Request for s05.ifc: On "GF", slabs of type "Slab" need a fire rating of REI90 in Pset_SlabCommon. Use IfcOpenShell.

First a look at what the model holds.

```python
import ifcopenshell
import ifcopenshell.util.element

model = ifcopenshell.open("s05.ifc")
print(model.schema)
storey = next(s for s in model.by_type("IfcBuildingStorey") if s.Name == "GF")
slabs = [e for e in ifcopenshell.util.element.get_decomposition(storey) if e.is_a("IfcSlab")]
seen = {}
for e in slabs:
    element_type = ifcopenshell.util.element.get_type(e)
    key = (element_type.Name if element_type != e and element_type else None, ifcopenshell.util.element.get_pset(e, "Pset_SlabCommon", "FireRating"))
    seen[key] = seen.get(key, 0) + 1
for (name, value), count in sorted(seen.items(), key=str):
    print(count, "x", name, "|", value)
```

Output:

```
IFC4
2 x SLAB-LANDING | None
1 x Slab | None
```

```python
import ifcopenshell
import ifcopenshell.api.pset
import ifcopenshell.util.element

model = ifcopenshell.open("s05.ifc")

storey = next(s for s in model.by_type("IfcBuildingStorey") if s.Name == "GF")
slabs = [e for e in ifcopenshell.util.element.get_decomposition(storey) if e.is_a("IfcSlab")]

count = 0
for e in slabs:
    element_type = ifcopenshell.util.element.get_type(e)
    if element_type in (None, e) or element_type.Name != "Slab":
        continue
    # add_pset returns the element's existing set when there is one.
    pset = ifcopenshell.api.pset.add_pset(model, product=e, name="Pset_SlabCommon")
    ifcopenshell.api.pset.edit_pset(model, pset=pset, properties={"FireRating": "REI90"})
    count += 1

print(count, "slabs updated")

model.write("s05_updated.ifc")
```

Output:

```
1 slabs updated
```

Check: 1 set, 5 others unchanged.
